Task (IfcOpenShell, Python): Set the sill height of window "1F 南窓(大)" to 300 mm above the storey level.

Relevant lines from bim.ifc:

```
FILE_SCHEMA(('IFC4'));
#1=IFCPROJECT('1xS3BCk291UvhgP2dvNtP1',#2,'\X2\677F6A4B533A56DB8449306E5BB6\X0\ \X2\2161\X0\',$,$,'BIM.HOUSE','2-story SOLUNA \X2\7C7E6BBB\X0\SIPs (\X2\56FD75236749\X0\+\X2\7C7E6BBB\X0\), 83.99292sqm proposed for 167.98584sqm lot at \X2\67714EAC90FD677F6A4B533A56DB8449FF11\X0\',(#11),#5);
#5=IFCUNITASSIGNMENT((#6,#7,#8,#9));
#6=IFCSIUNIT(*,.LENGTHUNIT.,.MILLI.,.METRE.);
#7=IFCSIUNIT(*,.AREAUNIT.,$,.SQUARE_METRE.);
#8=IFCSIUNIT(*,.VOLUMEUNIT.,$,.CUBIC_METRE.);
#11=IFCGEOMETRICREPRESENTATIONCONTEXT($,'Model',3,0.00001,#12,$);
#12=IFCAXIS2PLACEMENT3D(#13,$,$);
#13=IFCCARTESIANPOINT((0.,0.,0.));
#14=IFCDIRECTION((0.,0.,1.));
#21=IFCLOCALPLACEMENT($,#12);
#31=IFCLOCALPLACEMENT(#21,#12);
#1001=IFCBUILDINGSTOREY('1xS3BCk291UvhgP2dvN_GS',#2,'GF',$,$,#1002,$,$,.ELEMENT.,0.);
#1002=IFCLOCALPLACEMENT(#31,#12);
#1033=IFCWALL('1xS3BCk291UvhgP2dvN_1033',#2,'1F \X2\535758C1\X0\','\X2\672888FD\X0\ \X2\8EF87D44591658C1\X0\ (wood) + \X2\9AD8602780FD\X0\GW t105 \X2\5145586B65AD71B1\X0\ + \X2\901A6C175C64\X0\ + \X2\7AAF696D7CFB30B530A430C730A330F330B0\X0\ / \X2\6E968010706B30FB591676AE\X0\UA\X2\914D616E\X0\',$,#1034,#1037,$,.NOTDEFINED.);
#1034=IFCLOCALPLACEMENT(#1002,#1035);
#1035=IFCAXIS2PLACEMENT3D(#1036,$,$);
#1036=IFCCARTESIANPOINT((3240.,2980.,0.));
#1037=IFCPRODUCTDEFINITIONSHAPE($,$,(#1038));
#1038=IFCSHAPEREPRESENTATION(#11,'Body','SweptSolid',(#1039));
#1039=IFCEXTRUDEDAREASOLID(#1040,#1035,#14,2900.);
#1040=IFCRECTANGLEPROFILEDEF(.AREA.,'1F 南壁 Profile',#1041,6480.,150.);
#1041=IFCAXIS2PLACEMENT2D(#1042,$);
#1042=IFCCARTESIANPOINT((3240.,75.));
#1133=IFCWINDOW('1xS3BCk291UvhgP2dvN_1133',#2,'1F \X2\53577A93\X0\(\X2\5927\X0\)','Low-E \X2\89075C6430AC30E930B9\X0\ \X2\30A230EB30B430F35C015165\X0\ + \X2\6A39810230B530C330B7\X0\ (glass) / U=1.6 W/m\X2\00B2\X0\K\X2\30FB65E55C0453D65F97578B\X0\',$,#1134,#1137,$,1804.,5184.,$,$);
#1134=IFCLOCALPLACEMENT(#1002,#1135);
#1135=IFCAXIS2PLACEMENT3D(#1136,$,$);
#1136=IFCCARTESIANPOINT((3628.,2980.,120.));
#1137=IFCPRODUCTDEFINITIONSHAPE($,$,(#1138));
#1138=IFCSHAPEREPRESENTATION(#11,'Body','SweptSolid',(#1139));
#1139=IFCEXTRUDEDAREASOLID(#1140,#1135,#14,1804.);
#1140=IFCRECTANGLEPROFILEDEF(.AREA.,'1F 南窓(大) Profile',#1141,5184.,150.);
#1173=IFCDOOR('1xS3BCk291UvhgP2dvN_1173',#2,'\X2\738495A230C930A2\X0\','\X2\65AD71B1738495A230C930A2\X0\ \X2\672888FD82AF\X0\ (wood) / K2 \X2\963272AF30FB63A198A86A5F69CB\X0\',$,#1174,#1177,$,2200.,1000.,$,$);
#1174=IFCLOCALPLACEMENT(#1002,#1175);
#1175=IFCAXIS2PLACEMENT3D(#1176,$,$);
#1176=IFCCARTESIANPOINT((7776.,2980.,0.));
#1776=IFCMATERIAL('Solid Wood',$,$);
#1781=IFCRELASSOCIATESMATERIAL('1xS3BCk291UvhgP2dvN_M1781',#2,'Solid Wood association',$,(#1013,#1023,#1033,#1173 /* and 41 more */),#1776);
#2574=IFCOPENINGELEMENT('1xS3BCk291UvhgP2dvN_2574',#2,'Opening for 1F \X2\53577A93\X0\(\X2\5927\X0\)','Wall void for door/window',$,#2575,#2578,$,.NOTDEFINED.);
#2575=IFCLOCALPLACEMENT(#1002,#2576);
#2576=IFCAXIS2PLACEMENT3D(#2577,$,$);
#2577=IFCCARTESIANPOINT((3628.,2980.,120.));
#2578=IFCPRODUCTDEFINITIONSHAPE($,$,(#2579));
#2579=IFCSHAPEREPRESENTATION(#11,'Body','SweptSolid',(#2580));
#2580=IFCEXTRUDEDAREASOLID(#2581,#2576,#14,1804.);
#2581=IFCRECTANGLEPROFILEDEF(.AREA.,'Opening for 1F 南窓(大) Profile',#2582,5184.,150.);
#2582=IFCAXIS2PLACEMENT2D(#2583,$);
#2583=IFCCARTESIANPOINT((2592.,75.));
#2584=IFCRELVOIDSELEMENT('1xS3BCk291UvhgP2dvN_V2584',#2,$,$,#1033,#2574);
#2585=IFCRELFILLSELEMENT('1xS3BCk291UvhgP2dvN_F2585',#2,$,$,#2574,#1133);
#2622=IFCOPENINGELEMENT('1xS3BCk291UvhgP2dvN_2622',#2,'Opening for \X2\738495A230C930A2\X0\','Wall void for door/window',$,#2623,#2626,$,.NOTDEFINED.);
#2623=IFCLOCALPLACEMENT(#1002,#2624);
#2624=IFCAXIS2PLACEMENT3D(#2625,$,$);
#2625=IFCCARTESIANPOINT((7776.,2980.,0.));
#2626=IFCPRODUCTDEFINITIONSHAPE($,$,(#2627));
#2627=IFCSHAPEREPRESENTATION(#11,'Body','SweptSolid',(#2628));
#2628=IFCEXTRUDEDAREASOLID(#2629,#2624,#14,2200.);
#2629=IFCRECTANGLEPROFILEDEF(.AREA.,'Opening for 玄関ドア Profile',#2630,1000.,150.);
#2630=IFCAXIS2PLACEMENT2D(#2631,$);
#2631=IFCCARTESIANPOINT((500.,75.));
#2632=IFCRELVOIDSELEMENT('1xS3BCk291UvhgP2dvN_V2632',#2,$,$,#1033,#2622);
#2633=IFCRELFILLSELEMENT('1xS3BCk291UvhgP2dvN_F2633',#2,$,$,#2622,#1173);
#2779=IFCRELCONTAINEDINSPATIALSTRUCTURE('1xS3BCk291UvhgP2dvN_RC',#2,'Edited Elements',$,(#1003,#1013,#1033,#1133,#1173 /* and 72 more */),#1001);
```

```python
import numpy as np
import ifcopenshell
import ifcopenshell.api.geometry
import ifcopenshell.geom
import ifcopenshell.util.element
import ifcopenshell.util.placement
import ifcopenshell.util.shape
import ifcopenshell.util.unit

model = ifcopenshell.open("bim.ifc")
unit_scale = ifcopenshell.util.unit.calculate_unit_scale(model)

window = model.by_guid("1xS3BCk291UvhgP2dvN_1133")
opening = window.FillsVoids[0].RelatingOpeningElement
storey = ifcopenshell.util.element.get_container(window, ifc_class="IfcBuildingStorey")
level = ifcopenshell.util.placement.get_local_placement(storey.ObjectPlacement)[2, 3]

# The opening's origin need not be at the sill, so measure its lowest point.
shape = ifcopenshell.geom.create_shape(ifcopenshell.geom.settings(), opening)
bottom = ifcopenshell.util.shape.get_shape_bottom_elevation(shape, shape.geometry) / unit_scale
dz = level + 300.0 - bottom

shift = np.array([0.0, 0.0, dz])
# The window is not placed relative to its opening, so move both.
for product in (opening, window):
    matrix = ifcopenshell.util.placement.get_local_placement(product.ObjectPlacement)
    matrix[:3, 3] += shift
    ifcopenshell.api.geometry.edit_object_placement(model, product=product, matrix=matrix, is_si=False)

print(f"moved by {dz * unit_scale:+.3f} m")

model.write("bim_edited.ifc")
```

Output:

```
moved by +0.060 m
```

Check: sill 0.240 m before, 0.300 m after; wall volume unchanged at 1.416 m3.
